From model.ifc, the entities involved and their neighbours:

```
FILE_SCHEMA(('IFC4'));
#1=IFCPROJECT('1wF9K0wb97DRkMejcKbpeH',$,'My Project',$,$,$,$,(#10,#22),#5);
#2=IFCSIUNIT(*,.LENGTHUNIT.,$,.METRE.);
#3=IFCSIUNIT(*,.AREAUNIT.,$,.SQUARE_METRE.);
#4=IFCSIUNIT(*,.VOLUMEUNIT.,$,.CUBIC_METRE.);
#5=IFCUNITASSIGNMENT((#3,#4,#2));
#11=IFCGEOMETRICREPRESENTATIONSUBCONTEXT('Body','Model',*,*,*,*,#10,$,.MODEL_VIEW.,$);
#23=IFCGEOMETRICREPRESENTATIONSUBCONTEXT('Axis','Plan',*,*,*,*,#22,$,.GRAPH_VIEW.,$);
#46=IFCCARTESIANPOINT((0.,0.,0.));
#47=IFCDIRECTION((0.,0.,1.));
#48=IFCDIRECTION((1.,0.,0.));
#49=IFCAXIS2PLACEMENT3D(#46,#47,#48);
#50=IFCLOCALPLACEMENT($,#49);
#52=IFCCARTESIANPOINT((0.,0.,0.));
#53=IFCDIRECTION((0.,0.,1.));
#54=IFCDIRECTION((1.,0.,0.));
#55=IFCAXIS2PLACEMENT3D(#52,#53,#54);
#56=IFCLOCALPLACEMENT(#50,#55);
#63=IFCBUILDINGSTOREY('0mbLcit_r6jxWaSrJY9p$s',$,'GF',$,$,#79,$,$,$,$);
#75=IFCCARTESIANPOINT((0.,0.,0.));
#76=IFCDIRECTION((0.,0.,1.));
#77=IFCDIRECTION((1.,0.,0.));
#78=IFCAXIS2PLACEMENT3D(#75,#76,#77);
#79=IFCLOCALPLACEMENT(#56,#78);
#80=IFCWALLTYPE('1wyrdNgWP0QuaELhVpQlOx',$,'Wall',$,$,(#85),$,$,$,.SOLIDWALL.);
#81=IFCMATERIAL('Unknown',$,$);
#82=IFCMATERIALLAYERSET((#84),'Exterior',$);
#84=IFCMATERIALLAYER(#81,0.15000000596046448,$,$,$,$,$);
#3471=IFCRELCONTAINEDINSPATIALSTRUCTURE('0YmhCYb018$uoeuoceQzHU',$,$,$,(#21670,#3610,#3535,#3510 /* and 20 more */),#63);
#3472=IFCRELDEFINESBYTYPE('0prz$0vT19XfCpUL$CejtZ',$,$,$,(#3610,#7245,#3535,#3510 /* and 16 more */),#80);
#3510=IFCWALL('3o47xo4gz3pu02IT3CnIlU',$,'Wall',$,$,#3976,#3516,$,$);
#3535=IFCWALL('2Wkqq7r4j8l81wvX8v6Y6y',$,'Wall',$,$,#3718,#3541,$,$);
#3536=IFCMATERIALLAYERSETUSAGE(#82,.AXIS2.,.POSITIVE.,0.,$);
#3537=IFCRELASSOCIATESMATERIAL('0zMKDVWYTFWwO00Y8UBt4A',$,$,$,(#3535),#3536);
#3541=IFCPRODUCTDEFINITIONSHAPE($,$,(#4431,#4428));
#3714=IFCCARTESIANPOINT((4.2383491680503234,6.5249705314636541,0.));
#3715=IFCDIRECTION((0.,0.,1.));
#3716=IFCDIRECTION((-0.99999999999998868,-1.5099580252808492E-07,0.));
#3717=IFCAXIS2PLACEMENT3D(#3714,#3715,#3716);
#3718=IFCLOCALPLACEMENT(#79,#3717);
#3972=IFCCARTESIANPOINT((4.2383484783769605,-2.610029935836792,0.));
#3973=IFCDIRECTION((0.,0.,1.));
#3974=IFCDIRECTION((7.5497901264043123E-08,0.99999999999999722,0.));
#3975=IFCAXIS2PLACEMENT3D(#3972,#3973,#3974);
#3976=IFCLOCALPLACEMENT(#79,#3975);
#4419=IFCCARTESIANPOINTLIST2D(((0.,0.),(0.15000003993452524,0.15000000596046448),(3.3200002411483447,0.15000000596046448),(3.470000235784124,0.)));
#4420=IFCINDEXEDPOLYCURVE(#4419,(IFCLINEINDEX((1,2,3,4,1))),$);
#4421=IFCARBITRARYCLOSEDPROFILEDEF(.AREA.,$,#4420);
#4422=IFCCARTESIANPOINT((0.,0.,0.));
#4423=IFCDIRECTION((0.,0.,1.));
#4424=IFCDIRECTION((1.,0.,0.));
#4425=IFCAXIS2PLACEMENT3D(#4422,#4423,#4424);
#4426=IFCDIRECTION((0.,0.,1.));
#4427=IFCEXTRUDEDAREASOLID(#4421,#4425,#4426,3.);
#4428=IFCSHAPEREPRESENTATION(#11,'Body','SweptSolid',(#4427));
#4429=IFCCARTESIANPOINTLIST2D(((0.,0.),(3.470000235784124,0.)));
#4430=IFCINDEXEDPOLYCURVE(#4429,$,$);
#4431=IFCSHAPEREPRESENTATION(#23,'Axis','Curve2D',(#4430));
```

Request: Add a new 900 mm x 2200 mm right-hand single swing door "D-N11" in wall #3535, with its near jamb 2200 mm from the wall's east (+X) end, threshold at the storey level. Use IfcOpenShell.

```python
import numpy as np
import ifcopenshell
import ifcopenshell.api.feature
import ifcopenshell.api.geometry
import ifcopenshell.api.root
import ifcopenshell.api.spatial
import ifcopenshell.geom
import ifcopenshell.util.element
import ifcopenshell.util.placement
import ifcopenshell.util.representation
import ifcopenshell.util.shape
import ifcopenshell.util.unit

model = ifcopenshell.open("model.ifc")
unit_scale = ifcopenshell.util.unit.calculate_unit_scale(model)
settings = ifcopenshell.geom.settings()


def volume(element):
    """Net volume in cubic metres, openings subtracted."""
    shape = ifcopenshell.geom.create_shape(settings, element)
    return ifcopenshell.util.shape.get_volume(shape.geometry)


wall = model.by_guid("2Wkqq7r4j8l81wvX8v6Y6y")
storey = ifcopenshell.util.element.get_container(wall, ifc_class="IfcBuildingStorey")
context = ifcopenshell.util.representation.get_context(model, "Model", "Body", "MODEL_VIEW")
before = volume(wall)

width, height, from_end, sill = 0.9, 2.2, 2.2, 0.0  # metres

# The wall runs along its own X axis, and the end named is its -X end.
wall_shape = ifcopenshell.geom.create_shape(settings, wall)
x, y, z = ifcopenshell.util.shape.get_vertices(wall_shape.geometry).T
start = x.min() + from_end
face, thickness = float(y.min()), float(y.max() - y.min())
wall_matrix = ifcopenshell.util.placement.get_local_placement(wall.ObjectPlacement)
level = ifcopenshell.util.placement.get_local_placement(storey.ObjectPlacement)[2, 3]


def in_wall(x, y):
    """Placement at x, y metres in the wall's axes, at sill height."""
    matrix = wall_matrix.copy()
    matrix[:, 3] = wall_matrix @ np.array([x / unit_scale, y / unit_scale, 0.0, 1.0])
    matrix[2, 3] = level + sill / unit_scale
    return matrix


# Opening: a box that overshoots both wall faces by 50 mm.
opening = ifcopenshell.api.root.create_entity(model, ifc_class="IfcOpeningElement", predefined_type="OPENING")
box = ifcopenshell.api.geometry.add_wall_representation(
    model, context=context, length=width, height=height, thickness=thickness + 0.1
)
ifcopenshell.api.geometry.assign_representation(model, product=opening, representation=box)
ifcopenshell.api.geometry.edit_object_placement(model, product=opening, matrix=in_wall(start, face - 0.05), is_si=False)
ifcopenshell.api.feature.add_feature(model, feature=opening, element=wall)

door = ifcopenshell.api.root.create_entity(model, ifc_class="IfcDoor", name="D-N11", predefined_type="DOOR")
door.OverallWidth, door.OverallHeight = width / unit_scale, height / unit_scale
door.OperationType = "SINGLE_SWING_RIGHT"
body = ifcopenshell.api.geometry.add_door_representation(
    model,
    context=context,
    overall_width=door.OverallWidth,
    overall_height=door.OverallHeight,
    operation_type="SINGLE_SWING_RIGHT",
    lining_properties={"LiningDepth": thickness / unit_scale, "ThresholdDepth": thickness / unit_scale},
)
ifcopenshell.api.geometry.assign_representation(model, product=door, representation=body)
ifcopenshell.api.spatial.assign_container(model, products=[door], relating_structure=storey)
ifcopenshell.api.feature.add_filling(model, opening=opening, element=door)

# The lining spans the wall, so the door starts at the wall face.
ifcopenshell.api.geometry.edit_object_placement(model, product=door, matrix=in_wall(start, face), is_si=False)

after = volume(wall)

print(f"wall volume {before:.3f} -> {after:.3f} m3")

model.write("model_edited.ifc")
```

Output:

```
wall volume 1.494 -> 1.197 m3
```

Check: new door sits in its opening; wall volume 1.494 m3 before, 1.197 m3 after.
